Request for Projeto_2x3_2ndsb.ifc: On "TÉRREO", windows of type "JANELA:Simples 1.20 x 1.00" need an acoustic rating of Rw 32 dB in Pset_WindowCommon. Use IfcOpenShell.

First a look at what the model holds.

```python
import ifcopenshell
import ifcopenshell.util.element

model = ifcopenshell.open("Projeto_2x3_2ndsb.ifc")
print(model.schema)
storey = next(s for s in model.by_type("IfcBuildingStorey") if s.Name == "TÉRREO")
windows = [e for e in ifcopenshell.util.element.get_decomposition(storey) if e.is_a("IfcWindow")]
seen = {}
for e in windows:
    element_type = ifcopenshell.util.element.get_type(e)
    key = (element_type.Name if element_type != e and element_type else None, ifcopenshell.util.element.get_pset(e, "Pset_WindowCommon", "AcousticRating"))
    seen[key] = seen.get(key, 0) + 1
for (name, value), count in sorted(seen.items(), key=str):
    print(count, "x", name, "|", value)
```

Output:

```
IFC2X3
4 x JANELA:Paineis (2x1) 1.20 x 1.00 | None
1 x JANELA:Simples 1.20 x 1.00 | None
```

```python
import ifcopenshell
import ifcopenshell.api.pset
import ifcopenshell.util.element

model = ifcopenshell.open("Projeto_2x3_2ndsb.ifc")

storey = next(s for s in model.by_type("IfcBuildingStorey") if s.Name == "TÉRREO")
windows = [e for e in ifcopenshell.util.element.get_decomposition(storey) if e.is_a("IfcWindow")]

count = 0
for e in windows:
    element_type = ifcopenshell.util.element.get_type(e)
    if element_type in (None, e) or element_type.Name != "JANELA:Simples 1.20 x 1.00":
        continue
    # add_pset returns the element's existing set when there is one.
    pset = ifcopenshell.api.pset.add_pset(model, product=e, name="Pset_WindowCommon")
    ifcopenshell.api.pset.edit_pset(model, pset=pset, properties={"AcousticRating": "Rw 32 dB"})
    count += 1

print(count, "windows updated")

model.write("Projeto_2x3_2ndsb_edited.ifc")
```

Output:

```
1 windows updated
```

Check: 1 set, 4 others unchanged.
